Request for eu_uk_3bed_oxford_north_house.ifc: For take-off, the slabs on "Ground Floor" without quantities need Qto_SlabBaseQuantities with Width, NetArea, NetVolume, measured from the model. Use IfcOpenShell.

First a look at what the model holds.

```python
import ifcopenshell
import ifcopenshell.util.element
import ifcopenshell.util.unit

model = ifcopenshell.open("eu_uk_3bed_oxford_north_house.ifc")
print(model.schema)
for unit_type in ("LENGTHUNIT", "AREAUNIT", "VOLUMEUNIT"):
    print(unit_type, ifcopenshell.util.unit.calculate_unit_scale(model, unit_type))
storey = next(s for s in model.by_type("IfcBuildingStorey") if s.Name == "Ground Floor")
slabs = [e for e in ifcopenshell.util.element.get_decomposition(storey) if e.is_a("IfcSlab")]
for e in sorted(slabs, key=lambda e: e.id()):
    print(e.id(), e.is_a(), e.Name, list(ifcopenshell.util.element.get_psets(e, qtos_only=True)), sep=" | ")
```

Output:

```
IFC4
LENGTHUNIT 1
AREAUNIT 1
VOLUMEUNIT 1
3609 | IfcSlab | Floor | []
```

```python
import ifcopenshell
import ifcopenshell.api.pset
import ifcopenshell.geom
import ifcopenshell.util.element
import ifcopenshell.util.shape
import ifcopenshell.util.unit

model = ifcopenshell.open("eu_uk_3bed_oxford_north_house.ifc")
unit_scale = ifcopenshell.util.unit.calculate_unit_scale(model)
area_scale = ifcopenshell.util.unit.calculate_unit_scale(model, "AREAUNIT")
volume_scale = ifcopenshell.util.unit.calculate_unit_scale(model, "VOLUMEUNIT")
settings = ifcopenshell.geom.settings()

storey = next(s for s in model.by_type("IfcBuildingStorey") if s.Name == "Ground Floor")
slabs = [e for e in ifcopenshell.util.element.get_decomposition(storey) if e.is_a("IfcSlab")]

for e in sorted(slabs, key=lambda e: e.id()):
    if ifcopenshell.util.element.get_psets(e, qtos_only=True, should_inherit=False):
        continue
    # Geometry comes back in metres, in the element's own axes.
    shape = ifcopenshell.geom.create_shape(settings, e)
    values = {
        "Width": ifcopenshell.util.shape.get_z(shape.geometry) / unit_scale,
        "NetArea": ifcopenshell.util.shape.get_footprint_area(shape.geometry) / area_scale,
        "NetVolume": ifcopenshell.util.shape.get_volume(shape.geometry) / volume_scale,
    }
    qto = ifcopenshell.api.pset.add_qto(model, product=e, name="Qto_SlabBaseQuantities")
    ifcopenshell.api.pset.edit_qto(model, qto=qto, properties=values)
    print(e.id(), {k: round(v, 3) for k, v in values.items()})

model.write("eu_uk_3bed_oxford_north_house_v2.ifc")
```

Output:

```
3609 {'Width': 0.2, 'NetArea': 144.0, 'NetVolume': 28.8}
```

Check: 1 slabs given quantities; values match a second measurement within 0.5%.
